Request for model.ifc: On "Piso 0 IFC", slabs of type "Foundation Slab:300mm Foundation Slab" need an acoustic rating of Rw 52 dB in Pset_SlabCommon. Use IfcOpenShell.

First a look at what the model holds.

```python
import ifcopenshell
import ifcopenshell.util.element

model = ifcopenshell.open("model.ifc")
print(model.schema)
storey = next(s for s in model.by_type("IfcBuildingStorey") if s.Name == "Piso 0 IFC")
slabs = [e for e in ifcopenshell.util.element.get_decomposition(storey) if e.is_a("IfcSlab")]
seen = {}
for e in slabs:
    element_type = ifcopenshell.util.element.get_type(e)
    key = (element_type.Name if element_type != e and element_type else None, ifcopenshell.util.element.get_pset(e, "Pset_SlabCommon", "AcousticRating"))
    seen[key] = seen.get(key, 0) + 1
for (name, value), count in sorted(seen.items(), key=str):
    print(count, "x", name, "|", value)
```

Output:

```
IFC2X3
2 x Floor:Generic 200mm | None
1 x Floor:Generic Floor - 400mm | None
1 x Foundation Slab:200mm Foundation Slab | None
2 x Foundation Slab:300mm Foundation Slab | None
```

```python
import ifcopenshell
import ifcopenshell.api.pset
import ifcopenshell.util.element

model = ifcopenshell.open("model.ifc")

storey = next(s for s in model.by_type("IfcBuildingStorey") if s.Name == "Piso 0 IFC")
slabs = [e for e in ifcopenshell.util.element.get_decomposition(storey) if e.is_a("IfcSlab")]

count = 0
for e in slabs:
    element_type = ifcopenshell.util.element.get_type(e)
    if element_type in (None, e) or element_type.Name != "Foundation Slab:300mm Foundation Slab":
        continue
    # add_pset returns the element's existing set when there is one.
    pset = ifcopenshell.api.pset.add_pset(model, product=e, name="Pset_SlabCommon")
    ifcopenshell.api.pset.edit_pset(model, pset=pset, properties={"AcousticRating": "Rw 52 dB"})
    count += 1

print(count, "slabs updated")

model.write("model_v2.ifc")
```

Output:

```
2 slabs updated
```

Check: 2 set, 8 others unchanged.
